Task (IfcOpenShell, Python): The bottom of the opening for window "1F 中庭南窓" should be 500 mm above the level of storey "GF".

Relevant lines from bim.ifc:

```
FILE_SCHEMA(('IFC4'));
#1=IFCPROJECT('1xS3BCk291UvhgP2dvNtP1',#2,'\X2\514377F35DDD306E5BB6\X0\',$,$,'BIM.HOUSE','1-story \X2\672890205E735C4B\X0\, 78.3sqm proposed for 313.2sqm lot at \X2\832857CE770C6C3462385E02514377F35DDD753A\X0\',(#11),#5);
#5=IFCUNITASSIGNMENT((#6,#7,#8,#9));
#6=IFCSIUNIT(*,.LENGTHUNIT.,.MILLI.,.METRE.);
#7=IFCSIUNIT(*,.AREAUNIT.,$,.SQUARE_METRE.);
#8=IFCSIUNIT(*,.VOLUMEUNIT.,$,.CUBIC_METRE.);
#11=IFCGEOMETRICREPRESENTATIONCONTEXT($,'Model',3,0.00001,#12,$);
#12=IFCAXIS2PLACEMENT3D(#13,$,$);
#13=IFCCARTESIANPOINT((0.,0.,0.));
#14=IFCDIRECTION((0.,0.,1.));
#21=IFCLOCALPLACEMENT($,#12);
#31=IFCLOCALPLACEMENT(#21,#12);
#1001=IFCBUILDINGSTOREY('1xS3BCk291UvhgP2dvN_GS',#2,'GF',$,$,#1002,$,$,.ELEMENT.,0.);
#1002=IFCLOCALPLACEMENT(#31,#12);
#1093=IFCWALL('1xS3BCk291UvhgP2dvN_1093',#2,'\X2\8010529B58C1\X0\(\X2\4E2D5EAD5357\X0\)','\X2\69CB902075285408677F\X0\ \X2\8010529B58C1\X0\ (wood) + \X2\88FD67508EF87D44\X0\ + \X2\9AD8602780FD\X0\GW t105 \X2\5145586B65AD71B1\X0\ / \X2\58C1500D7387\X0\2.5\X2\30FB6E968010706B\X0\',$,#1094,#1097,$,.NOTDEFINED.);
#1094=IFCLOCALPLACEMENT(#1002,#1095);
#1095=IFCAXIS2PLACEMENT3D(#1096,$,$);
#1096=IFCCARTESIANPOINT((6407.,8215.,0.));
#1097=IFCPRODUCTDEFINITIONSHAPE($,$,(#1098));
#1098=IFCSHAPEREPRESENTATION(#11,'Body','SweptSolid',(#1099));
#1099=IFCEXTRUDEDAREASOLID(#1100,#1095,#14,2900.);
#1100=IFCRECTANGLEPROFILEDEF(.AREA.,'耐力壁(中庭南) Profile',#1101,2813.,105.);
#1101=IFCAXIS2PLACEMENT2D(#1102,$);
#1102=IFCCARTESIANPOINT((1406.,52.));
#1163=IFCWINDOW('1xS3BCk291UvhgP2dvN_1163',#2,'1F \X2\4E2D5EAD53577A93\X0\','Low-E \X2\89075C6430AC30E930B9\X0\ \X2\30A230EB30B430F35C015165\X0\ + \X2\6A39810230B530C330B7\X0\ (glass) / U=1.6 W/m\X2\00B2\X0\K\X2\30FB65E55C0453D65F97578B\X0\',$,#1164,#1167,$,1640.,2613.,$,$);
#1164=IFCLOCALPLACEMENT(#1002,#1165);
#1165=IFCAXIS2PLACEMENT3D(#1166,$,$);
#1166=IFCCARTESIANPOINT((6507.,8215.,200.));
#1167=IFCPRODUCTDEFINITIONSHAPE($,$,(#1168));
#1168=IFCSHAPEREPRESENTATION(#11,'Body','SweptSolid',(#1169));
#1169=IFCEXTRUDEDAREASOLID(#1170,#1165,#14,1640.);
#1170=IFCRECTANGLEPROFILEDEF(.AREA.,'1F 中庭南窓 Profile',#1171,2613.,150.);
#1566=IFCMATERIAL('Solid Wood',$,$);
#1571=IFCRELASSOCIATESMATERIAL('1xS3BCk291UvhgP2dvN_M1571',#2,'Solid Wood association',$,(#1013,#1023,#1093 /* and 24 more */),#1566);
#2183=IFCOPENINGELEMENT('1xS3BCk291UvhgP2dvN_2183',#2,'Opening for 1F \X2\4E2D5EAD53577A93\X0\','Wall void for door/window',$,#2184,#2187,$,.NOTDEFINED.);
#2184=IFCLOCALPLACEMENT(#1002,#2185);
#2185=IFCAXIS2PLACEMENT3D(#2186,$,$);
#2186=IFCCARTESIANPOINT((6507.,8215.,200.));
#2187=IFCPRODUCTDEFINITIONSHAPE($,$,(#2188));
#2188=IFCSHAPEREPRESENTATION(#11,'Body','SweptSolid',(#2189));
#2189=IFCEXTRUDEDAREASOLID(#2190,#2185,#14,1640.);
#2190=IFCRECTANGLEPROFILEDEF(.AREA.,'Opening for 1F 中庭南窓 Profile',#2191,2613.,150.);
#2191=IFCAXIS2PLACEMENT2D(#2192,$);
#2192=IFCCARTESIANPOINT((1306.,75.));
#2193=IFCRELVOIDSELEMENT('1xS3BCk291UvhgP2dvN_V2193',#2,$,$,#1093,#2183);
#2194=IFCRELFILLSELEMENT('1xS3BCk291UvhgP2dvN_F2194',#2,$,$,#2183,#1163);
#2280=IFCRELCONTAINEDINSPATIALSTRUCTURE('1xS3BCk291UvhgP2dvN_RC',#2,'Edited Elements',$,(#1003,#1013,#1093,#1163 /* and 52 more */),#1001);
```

```python
import numpy as np
import ifcopenshell
import ifcopenshell.api.geometry
import ifcopenshell.geom
import ifcopenshell.util.element
import ifcopenshell.util.placement
import ifcopenshell.util.shape
import ifcopenshell.util.unit

model = ifcopenshell.open("bim.ifc")
unit_scale = ifcopenshell.util.unit.calculate_unit_scale(model)

window = model.by_guid("1xS3BCk291UvhgP2dvN_1163")
opening = window.FillsVoids[0].RelatingOpeningElement
storey = ifcopenshell.util.element.get_container(window, ifc_class="IfcBuildingStorey")
level = ifcopenshell.util.placement.get_local_placement(storey.ObjectPlacement)[2, 3]

# The opening's origin need not be at the sill, so measure its lowest point.
shape = ifcopenshell.geom.create_shape(ifcopenshell.geom.settings(), opening)
bottom = ifcopenshell.util.shape.get_shape_bottom_elevation(shape, shape.geometry) / unit_scale
dz = level + 500.0 - bottom

shift = np.array([0.0, 0.0, dz])
# The window is not placed relative to its opening, so move both.
for product in (opening, window):
    matrix = ifcopenshell.util.placement.get_local_placement(product.ObjectPlacement)
    matrix[:3, 3] += shift
    ifcopenshell.api.geometry.edit_object_placement(model, product=product, matrix=matrix, is_si=False)

print(f"moved by {dz * unit_scale:+.3f} m")

model.write("bim-out.ifc")
```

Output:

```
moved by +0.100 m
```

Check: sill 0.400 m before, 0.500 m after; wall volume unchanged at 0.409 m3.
